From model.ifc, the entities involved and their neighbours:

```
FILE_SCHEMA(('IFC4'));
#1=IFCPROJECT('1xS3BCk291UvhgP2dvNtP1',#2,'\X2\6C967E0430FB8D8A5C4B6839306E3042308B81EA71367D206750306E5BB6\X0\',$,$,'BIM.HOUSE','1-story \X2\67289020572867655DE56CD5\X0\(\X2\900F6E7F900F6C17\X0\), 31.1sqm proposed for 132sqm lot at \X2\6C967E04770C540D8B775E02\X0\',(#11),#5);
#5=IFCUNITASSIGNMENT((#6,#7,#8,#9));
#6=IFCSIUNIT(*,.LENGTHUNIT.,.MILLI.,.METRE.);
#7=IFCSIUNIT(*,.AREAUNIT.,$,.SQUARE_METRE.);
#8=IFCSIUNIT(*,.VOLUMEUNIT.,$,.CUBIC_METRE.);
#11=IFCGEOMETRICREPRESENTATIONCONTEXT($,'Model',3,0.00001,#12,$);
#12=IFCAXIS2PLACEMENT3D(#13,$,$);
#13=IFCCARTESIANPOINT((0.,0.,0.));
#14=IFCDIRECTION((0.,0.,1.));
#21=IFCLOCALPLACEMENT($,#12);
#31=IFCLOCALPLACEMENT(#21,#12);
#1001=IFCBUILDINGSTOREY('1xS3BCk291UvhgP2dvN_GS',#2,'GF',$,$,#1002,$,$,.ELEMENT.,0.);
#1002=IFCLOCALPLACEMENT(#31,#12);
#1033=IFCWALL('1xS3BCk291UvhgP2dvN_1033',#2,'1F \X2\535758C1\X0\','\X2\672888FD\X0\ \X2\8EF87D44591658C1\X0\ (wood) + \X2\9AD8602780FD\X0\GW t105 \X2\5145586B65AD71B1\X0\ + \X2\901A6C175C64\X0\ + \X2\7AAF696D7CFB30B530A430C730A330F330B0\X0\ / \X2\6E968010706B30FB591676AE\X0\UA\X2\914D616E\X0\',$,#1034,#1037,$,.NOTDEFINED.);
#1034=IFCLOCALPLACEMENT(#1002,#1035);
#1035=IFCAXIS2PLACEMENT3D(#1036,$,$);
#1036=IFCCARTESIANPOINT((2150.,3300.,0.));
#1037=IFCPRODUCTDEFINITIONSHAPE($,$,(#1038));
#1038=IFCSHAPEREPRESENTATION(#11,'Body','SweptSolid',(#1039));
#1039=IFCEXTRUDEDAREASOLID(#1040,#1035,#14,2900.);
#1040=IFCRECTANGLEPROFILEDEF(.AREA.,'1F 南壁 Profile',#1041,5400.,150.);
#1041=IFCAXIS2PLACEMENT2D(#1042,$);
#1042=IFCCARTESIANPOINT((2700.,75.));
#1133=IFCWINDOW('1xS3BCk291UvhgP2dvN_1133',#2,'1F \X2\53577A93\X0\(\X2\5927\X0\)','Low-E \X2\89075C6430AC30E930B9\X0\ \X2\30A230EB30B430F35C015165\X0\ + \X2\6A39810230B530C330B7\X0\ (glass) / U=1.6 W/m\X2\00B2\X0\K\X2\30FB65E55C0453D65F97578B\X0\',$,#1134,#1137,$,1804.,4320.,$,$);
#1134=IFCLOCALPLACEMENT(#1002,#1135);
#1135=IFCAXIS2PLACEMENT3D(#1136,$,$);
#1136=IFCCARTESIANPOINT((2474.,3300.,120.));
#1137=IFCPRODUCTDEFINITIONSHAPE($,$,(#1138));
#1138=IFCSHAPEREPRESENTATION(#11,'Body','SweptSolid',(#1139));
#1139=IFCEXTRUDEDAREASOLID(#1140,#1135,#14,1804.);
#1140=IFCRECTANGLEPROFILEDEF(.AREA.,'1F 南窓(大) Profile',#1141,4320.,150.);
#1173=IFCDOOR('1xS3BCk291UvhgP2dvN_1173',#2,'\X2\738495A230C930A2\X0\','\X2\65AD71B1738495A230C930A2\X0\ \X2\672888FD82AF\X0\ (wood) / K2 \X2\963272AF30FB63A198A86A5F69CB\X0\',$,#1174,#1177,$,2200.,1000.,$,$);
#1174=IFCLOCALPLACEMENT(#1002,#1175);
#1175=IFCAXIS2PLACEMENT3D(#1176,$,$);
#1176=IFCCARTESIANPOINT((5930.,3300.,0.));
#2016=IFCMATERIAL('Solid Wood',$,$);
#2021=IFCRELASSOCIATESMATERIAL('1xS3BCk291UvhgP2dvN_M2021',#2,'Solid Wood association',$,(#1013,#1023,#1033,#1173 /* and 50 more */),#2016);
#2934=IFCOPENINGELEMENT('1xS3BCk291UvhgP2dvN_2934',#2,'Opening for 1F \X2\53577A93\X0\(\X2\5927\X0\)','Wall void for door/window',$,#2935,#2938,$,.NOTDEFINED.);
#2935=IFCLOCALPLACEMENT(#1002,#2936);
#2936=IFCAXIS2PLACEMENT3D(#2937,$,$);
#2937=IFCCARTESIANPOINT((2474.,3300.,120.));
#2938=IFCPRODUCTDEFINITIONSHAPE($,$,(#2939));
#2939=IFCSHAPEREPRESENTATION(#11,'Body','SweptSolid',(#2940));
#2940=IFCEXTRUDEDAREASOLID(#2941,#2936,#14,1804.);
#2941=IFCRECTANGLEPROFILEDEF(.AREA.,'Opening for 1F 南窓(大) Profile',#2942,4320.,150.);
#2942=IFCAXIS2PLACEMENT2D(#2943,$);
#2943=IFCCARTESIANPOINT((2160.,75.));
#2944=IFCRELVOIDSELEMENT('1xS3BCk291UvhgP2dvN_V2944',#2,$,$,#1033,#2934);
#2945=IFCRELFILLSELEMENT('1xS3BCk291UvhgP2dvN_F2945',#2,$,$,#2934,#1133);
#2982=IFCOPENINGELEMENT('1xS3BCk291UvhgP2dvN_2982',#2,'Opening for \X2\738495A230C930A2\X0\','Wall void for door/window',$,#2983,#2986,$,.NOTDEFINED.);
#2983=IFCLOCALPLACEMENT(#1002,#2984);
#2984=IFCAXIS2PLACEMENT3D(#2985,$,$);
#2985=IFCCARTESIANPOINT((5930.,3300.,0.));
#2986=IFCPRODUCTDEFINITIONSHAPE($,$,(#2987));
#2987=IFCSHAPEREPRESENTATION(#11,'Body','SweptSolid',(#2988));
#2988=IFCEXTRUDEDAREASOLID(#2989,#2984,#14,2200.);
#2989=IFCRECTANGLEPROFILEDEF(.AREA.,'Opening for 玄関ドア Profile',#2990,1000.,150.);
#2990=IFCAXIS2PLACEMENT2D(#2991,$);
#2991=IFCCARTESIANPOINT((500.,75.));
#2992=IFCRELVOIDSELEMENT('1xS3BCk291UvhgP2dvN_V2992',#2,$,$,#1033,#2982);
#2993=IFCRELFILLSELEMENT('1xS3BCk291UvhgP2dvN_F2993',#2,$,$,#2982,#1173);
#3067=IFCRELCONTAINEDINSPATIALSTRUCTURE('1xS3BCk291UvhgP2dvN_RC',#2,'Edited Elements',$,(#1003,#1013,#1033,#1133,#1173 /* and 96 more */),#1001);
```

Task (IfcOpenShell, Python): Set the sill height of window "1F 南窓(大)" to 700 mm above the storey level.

```python
import numpy as np
import ifcopenshell
import ifcopenshell.api.geometry
import ifcopenshell.geom
import ifcopenshell.util.element
import ifcopenshell.util.placement
import ifcopenshell.util.shape
import ifcopenshell.util.unit

model = ifcopenshell.open("model.ifc")
unit_scale = ifcopenshell.util.unit.calculate_unit_scale(model)

window = model.by_guid("1xS3BCk291UvhgP2dvN_1133")
opening = window.FillsVoids[0].RelatingOpeningElement
storey = ifcopenshell.util.element.get_container(window, ifc_class="IfcBuildingStorey")
level = ifcopenshell.util.placement.get_local_placement(storey.ObjectPlacement)[2, 3]

# The opening's origin need not be at the sill, so measure its lowest point.
shape = ifcopenshell.geom.create_shape(ifcopenshell.geom.settings(), opening)
bottom = ifcopenshell.util.shape.get_shape_bottom_elevation(shape, shape.geometry) / unit_scale
dz = level + 700.0 - bottom

shift = np.array([0.0, 0.0, dz])
# The window is not placed relative to its opening, so move both.
for product in (opening, window):
    matrix = ifcopenshell.util.placement.get_local_placement(product.ObjectPlacement)
    matrix[:3, 3] += shift
    ifcopenshell.api.geometry.edit_object_placement(model, product=product, matrix=matrix, is_si=False)

print(f"moved by {dz * unit_scale:+.3f} m")

model.write("model_updated.ifc")
```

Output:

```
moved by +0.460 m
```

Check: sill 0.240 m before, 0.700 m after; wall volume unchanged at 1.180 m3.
